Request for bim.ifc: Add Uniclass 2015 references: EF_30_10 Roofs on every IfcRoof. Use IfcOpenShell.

First a look at what the model holds.

```python
import ifcopenshell

model = ifcopenshell.open("bim.ifc")
print(model.schema)
print("classifications:", [c.Name for c in model.by_type("IfcClassification")])
for ifc_class in ("IfcDoor", "IfcRoof", "IfcStair", "IfcWall", "IfcWindow"):
    print(ifc_class, len(model.by_type(ifc_class)))
```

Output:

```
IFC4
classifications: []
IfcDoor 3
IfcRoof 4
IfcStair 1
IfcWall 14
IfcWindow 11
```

```python
import ifcopenshell
import ifcopenshell.api.classification

model = ifcopenshell.open("bim.ifc")

system = ifcopenshell.api.classification.add_classification(model, classification="Uniclass 2015")

codes = {
    "IfcRoof": ("EF_30_10", "Roofs"),
}
for ifc_class, (code, name) in codes.items():
    products = model.by_type(ifc_class)
    ifcopenshell.api.classification.add_reference(
        model, products=products, classification=system, identification=code, name=name
    )
    print(code, len(products))

model.write("bim_updated.ifc")
```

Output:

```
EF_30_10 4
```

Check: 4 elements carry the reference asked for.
